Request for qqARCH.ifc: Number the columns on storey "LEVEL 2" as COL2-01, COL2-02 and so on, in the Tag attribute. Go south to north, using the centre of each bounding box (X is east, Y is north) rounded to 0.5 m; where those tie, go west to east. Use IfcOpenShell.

First a look at what the model holds.

```python
import ifcopenshell
import ifcopenshell.util.element
import ifcopenshell.util.placement

model = ifcopenshell.open("qqARCH.ifc")
print(model.schema)
storey = next(s for s in model.by_type("IfcBuildingStorey") if s.Name == "LEVEL 2")
columns = [e for e in ifcopenshell.util.element.get_decomposition(storey) if e.is_a("IfcColumn")]
for e in sorted(columns, key=lambda e: e.id()):
    origin = ifcopenshell.util.placement.get_local_placement(e.ObjectPlacement)[:3, 3]
    print(e.id(), e.Tag, e.Name, origin.round(2) + 0.0, sep=" | ")
```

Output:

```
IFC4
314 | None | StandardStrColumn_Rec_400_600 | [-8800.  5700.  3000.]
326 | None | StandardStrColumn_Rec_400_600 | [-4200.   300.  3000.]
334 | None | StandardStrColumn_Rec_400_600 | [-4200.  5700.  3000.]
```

```python
import ifcopenshell
import ifcopenshell.geom
import ifcopenshell.util.element
import ifcopenshell.util.shape

model = ifcopenshell.open("qqARCH.ifc")
settings = ifcopenshell.geom.settings()
settings.set("use-world-coords", True)


def centre(element):
    shape = ifcopenshell.geom.create_shape(settings, element)
    return ifcopenshell.util.shape.get_bbox_centroid(shape.geometry)


storey = next(s for s in model.by_type("IfcBuildingStorey") if s.Name == "LEVEL 2")
columns = [e for e in ifcopenshell.util.element.get_decomposition(storey) if e.is_a("IfcColumn")]

# Insertion points can sit at a corner or the storey origin, so sort by the geometry (in metres).
centres = {e: centre(e) for e in columns}
columns.sort(key=lambda e: (round(centres[e][1] / 0.5), centres[e][0]))

for i, e in enumerate(columns, start=1):
    number = f"COL2-{i:02d}"
    e.Tag = number
    print(e.id(), number)

model.write("qqARCH_updated.ifc")
```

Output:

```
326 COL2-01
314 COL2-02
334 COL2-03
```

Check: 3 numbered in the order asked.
